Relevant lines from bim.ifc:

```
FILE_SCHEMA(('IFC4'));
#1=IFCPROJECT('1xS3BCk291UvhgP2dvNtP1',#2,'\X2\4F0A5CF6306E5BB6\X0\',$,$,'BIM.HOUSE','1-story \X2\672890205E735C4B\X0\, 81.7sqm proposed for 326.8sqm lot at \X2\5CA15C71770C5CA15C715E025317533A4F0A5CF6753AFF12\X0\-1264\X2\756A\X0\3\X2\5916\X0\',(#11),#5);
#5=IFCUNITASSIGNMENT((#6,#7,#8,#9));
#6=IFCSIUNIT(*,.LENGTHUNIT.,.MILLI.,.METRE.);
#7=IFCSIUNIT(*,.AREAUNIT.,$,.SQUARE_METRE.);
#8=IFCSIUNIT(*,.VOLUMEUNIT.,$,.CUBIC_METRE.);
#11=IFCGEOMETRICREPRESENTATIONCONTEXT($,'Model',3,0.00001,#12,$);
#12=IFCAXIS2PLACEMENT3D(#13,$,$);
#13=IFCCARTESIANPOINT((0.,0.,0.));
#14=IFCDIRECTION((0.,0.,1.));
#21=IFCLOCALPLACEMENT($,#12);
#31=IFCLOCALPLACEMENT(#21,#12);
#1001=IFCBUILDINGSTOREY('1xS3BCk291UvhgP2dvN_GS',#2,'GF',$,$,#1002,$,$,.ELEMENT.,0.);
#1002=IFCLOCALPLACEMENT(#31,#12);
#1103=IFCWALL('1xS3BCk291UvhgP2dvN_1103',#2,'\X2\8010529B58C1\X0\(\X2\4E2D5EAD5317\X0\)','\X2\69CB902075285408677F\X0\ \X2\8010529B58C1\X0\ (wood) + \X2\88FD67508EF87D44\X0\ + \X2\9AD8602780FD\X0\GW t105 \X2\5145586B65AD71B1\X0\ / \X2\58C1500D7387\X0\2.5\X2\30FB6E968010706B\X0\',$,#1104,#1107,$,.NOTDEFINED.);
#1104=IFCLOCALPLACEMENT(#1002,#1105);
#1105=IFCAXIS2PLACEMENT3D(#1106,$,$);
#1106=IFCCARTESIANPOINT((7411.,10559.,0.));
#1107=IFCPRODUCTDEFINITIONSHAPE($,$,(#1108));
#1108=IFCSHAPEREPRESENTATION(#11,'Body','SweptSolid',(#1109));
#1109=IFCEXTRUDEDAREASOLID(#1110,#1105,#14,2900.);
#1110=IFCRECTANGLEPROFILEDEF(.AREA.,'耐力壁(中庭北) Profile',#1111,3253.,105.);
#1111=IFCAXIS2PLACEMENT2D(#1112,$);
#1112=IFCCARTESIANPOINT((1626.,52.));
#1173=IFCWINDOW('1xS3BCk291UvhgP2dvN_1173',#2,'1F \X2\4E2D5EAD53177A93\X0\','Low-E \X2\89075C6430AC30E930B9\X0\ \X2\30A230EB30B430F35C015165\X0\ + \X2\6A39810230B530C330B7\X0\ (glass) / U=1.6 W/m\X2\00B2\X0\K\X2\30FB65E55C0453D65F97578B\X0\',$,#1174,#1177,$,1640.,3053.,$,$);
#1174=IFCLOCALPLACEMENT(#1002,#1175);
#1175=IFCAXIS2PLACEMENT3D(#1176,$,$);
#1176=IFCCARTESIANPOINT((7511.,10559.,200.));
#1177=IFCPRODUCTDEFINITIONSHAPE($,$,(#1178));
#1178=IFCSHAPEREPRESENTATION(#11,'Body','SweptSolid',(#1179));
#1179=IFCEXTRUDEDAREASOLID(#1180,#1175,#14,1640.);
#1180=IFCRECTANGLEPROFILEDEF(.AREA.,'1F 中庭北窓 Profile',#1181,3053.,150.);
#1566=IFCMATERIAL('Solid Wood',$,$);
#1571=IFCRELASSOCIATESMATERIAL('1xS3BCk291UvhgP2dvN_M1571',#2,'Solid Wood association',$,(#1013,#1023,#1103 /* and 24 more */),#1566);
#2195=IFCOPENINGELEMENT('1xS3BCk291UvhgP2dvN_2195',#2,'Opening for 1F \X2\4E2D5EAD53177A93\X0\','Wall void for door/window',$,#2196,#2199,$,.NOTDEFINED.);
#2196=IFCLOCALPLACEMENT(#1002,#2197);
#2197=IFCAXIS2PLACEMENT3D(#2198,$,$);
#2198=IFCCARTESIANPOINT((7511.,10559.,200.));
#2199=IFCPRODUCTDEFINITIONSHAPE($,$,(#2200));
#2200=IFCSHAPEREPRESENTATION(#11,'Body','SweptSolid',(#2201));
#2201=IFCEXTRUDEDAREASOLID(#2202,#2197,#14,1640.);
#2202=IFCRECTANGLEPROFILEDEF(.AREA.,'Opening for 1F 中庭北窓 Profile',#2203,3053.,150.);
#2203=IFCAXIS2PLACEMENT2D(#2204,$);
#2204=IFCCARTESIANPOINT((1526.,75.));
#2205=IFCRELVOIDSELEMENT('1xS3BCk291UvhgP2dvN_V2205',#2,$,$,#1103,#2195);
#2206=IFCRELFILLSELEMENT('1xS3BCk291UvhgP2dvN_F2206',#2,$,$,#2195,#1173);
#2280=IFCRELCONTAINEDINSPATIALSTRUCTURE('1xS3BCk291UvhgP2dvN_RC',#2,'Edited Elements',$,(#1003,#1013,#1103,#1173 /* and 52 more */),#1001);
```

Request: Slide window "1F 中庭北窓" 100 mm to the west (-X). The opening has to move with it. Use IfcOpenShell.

```python
import ifcopenshell
import ifcopenshell.api.geometry
import ifcopenshell.util.placement
import ifcopenshell.util.unit

model = ifcopenshell.open("bim.ifc")
unit_scale = ifcopenshell.util.unit.calculate_unit_scale(model)

window = model.by_guid("1xS3BCk291UvhgP2dvN_1173")
opening = window.FillsVoids[0].RelatingOpeningElement
wall = opening.VoidsElements[0].RelatingBuildingElement

wall_matrix = ifcopenshell.util.placement.get_local_placement(wall.ObjectPlacement)
shift = wall_matrix[:3, 0] * -0.1 / unit_scale
before = ifcopenshell.util.placement.get_local_placement(window.ObjectPlacement)[:3, 3].copy()

# The window is not placed relative to its opening, so move both.
for product in (opening, window):
    matrix = ifcopenshell.util.placement.get_local_placement(product.ObjectPlacement)
    matrix[:3, 3] += shift
    ifcopenshell.api.geometry.edit_object_placement(model, product=product, matrix=matrix, is_si=False)

after = ifcopenshell.util.placement.get_local_placement(window.ObjectPlacement)[:3, 3]
print("window moved by", (after - before).round(3) + 0.0)

model.write("bim-out.ifc")
```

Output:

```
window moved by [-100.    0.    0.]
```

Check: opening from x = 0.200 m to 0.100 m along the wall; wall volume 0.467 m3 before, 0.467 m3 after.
